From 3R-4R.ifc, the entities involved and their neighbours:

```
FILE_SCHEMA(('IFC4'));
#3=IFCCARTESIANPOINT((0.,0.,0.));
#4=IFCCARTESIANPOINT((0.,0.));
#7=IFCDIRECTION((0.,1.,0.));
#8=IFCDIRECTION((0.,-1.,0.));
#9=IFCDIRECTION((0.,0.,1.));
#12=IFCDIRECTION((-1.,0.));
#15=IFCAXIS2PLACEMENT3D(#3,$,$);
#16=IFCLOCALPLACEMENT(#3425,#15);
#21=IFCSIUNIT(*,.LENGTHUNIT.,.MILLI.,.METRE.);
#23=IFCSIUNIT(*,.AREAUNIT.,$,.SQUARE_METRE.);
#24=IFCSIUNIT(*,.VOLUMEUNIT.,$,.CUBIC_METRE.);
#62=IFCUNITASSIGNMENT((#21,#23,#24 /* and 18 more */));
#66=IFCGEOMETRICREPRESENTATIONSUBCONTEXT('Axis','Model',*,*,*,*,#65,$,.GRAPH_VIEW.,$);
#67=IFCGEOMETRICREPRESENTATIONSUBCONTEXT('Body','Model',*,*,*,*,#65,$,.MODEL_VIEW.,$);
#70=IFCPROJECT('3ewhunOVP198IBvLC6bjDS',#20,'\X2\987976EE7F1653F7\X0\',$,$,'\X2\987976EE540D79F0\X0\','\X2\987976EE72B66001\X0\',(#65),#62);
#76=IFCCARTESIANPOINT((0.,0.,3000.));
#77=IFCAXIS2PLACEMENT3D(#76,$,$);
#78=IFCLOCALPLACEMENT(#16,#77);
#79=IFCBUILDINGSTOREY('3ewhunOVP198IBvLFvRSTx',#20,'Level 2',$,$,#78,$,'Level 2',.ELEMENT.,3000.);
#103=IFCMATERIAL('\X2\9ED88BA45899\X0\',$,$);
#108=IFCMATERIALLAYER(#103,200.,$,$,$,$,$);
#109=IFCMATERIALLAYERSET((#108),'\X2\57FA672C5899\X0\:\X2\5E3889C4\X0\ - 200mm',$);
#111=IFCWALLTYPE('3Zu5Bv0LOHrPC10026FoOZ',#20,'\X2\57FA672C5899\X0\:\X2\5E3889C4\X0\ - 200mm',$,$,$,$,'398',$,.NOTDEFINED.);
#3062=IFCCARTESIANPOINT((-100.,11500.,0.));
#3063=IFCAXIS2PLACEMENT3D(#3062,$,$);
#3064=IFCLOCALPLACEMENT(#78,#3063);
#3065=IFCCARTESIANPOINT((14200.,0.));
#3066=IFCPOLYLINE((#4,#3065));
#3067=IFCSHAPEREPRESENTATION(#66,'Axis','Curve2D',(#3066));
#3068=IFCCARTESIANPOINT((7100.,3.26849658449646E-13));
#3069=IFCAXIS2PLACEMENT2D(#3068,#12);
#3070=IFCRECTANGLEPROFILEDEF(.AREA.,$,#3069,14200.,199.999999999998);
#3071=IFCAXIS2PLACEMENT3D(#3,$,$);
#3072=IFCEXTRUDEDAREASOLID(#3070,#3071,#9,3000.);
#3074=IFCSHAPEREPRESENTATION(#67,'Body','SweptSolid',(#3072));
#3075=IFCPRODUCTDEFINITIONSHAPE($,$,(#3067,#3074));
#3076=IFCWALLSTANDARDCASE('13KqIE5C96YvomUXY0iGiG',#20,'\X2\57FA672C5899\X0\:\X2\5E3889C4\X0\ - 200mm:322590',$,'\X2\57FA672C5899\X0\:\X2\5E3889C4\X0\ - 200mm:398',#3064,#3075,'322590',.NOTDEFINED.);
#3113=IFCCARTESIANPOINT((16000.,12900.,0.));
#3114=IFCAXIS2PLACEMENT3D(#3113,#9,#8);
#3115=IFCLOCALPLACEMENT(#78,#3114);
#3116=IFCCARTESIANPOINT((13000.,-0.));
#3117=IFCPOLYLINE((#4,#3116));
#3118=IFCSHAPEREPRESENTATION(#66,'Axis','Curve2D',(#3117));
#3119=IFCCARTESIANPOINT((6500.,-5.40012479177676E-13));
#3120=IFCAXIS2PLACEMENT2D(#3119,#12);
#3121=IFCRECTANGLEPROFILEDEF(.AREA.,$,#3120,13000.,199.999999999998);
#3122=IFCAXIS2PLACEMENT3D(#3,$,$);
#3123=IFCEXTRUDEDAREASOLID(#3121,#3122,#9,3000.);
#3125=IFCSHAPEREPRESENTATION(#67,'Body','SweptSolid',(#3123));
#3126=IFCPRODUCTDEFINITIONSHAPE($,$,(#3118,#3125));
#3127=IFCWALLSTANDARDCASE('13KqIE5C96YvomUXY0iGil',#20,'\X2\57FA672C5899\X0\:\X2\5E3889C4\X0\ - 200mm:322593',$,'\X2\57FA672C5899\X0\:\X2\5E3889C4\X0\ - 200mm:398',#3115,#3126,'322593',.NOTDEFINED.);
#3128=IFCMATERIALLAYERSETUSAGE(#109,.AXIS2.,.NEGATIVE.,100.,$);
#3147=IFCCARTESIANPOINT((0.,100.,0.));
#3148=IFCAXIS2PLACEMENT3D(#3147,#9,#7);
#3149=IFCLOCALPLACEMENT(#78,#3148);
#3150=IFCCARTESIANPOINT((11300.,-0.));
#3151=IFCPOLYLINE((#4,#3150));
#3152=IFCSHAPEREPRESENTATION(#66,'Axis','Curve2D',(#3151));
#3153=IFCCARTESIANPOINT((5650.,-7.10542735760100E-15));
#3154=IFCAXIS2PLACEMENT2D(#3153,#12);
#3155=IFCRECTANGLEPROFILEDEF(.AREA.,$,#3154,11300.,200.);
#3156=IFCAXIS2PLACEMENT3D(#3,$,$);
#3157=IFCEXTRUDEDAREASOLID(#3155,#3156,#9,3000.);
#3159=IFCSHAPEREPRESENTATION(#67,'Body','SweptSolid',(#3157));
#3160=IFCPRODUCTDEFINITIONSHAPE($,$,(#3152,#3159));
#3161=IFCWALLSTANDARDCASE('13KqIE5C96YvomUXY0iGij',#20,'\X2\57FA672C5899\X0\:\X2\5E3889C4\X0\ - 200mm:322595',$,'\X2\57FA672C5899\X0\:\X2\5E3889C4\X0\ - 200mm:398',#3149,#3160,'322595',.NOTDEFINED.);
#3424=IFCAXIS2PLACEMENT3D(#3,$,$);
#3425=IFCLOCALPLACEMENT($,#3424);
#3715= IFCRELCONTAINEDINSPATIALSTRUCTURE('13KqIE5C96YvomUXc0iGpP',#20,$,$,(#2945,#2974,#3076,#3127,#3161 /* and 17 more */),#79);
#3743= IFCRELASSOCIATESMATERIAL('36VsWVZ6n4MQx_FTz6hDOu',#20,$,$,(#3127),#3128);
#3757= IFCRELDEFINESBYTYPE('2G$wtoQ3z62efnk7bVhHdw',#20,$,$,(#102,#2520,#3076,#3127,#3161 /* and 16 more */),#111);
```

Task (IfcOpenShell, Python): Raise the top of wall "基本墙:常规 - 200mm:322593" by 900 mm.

```python
import ifcopenshell
import ifcopenshell.geom
import ifcopenshell.util.representation
import ifcopenshell.util.shape

model = ifcopenshell.open("3R-4R.ifc")
settings = ifcopenshell.geom.settings()


def volume(element):
    """Net volume in cubic metres, openings subtracted."""
    shape = ifcopenshell.geom.create_shape(settings, element)
    return ifcopenshell.util.shape.get_volume(shape.geometry)


wall = model.by_guid("13KqIE5C96YvomUXY0iGil")
before = volume(wall)

body = ifcopenshell.util.representation.get_representation(wall, "Model", "Body")
solid = body.Items[0]
old_height = solid.Depth
solid.Depth += 900.0
after = volume(wall)

print(f"height {old_height:g} -> {solid.Depth:g}, volume {before:.3f} -> {after:.3f} m3")

model.write("3R-4R_rev.ifc")
```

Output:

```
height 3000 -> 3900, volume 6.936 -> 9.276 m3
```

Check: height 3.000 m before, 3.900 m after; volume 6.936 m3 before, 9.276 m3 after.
